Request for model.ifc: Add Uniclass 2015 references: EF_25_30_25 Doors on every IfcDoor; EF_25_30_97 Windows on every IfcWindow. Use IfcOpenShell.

First a look at what the model holds.

```python
import ifcopenshell

model = ifcopenshell.open("model.ifc")
print(model.schema)
print("classifications:", [c.Name for c in model.by_type("IfcClassification")])
for ifc_class in ("IfcDoor", "IfcRoof", "IfcStair", "IfcWall", "IfcWindow"):
    print(ifc_class, len(model.by_type(ifc_class)))
```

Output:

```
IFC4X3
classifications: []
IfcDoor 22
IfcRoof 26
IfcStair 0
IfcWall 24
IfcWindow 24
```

```python
import ifcopenshell
import ifcopenshell.api.classification

model = ifcopenshell.open("model.ifc")

system = ifcopenshell.api.classification.add_classification(model, classification="Uniclass 2015")

codes = {
    "IfcDoor": ("EF_25_30_25", "Doors"),
    "IfcWindow": ("EF_25_30_97", "Windows"),
}
for ifc_class, (code, name) in codes.items():
    products = model.by_type(ifc_class)
    ifcopenshell.api.classification.add_reference(
        model, products=products, classification=system, identification=code, name=name
    )
    print(code, len(products))

model.write("model_v2.ifc")
```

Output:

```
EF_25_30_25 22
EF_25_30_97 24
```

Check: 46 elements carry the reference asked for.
